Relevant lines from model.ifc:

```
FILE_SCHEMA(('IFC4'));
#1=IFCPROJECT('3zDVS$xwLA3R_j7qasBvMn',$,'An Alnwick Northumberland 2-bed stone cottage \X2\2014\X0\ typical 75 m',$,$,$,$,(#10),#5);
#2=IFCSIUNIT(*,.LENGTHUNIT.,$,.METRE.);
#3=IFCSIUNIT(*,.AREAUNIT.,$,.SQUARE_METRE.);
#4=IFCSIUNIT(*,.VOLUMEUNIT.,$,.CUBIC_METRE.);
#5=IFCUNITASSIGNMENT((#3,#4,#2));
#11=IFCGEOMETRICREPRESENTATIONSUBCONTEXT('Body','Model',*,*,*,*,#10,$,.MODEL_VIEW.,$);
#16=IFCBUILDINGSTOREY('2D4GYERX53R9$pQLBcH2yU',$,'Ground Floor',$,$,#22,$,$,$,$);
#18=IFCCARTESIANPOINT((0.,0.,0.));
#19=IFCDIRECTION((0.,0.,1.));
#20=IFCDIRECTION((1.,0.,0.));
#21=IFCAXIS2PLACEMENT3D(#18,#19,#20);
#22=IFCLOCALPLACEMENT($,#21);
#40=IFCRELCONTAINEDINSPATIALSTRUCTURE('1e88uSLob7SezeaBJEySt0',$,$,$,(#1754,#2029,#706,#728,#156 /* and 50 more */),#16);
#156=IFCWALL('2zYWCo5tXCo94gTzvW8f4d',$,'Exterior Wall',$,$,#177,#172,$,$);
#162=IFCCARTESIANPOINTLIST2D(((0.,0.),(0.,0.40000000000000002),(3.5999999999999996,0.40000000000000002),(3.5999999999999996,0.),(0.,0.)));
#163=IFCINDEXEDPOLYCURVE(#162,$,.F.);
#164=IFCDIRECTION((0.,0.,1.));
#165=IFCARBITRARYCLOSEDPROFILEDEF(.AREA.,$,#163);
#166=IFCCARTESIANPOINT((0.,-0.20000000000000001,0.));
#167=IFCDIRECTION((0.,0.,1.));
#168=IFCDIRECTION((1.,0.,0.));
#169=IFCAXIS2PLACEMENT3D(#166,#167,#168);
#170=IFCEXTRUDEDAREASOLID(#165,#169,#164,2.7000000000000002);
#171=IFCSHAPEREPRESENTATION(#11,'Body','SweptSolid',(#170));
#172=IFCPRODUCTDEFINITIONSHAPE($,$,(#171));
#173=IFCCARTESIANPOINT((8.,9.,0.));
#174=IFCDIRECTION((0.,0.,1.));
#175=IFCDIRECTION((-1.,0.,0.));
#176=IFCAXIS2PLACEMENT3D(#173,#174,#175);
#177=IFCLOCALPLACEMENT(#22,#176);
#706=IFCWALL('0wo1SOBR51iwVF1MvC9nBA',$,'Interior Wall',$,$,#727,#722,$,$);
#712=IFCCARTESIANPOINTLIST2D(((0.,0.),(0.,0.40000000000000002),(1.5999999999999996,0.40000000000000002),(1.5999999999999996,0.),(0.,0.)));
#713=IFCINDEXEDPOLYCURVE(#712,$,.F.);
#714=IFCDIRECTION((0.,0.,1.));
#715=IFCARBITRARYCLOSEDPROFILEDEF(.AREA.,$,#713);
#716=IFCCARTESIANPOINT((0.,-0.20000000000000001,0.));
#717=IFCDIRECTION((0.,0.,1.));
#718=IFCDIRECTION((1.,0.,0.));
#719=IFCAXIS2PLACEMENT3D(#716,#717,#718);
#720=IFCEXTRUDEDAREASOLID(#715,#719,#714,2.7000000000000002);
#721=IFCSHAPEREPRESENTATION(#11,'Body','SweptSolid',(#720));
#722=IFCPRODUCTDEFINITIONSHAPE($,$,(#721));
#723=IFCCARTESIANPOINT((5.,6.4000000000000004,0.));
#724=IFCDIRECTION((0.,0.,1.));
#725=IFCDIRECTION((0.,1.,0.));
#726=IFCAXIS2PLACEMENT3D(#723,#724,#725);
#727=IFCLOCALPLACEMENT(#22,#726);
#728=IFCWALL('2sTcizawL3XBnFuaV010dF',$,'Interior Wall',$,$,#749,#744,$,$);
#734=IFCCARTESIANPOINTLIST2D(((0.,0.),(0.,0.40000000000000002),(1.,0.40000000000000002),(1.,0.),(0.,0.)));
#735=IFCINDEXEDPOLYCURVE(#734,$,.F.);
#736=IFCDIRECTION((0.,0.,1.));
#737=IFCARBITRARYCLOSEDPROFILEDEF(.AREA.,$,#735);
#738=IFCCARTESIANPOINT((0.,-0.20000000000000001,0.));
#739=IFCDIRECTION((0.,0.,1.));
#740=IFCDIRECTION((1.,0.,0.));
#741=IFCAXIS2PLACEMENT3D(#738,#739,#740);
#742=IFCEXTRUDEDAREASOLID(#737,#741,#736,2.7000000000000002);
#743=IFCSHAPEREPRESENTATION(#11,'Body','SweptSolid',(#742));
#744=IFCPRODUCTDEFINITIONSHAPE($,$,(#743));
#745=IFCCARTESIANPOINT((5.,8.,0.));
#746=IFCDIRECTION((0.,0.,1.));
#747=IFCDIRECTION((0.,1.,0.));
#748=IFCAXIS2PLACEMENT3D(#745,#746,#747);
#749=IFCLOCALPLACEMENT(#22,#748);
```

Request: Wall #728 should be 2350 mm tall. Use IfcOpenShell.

```python
import ifcopenshell
import ifcopenshell.geom
import ifcopenshell.util.representation
import ifcopenshell.util.shape
import ifcopenshell.util.unit

model = ifcopenshell.open("model.ifc")
unit_scale = ifcopenshell.util.unit.calculate_unit_scale(model)
settings = ifcopenshell.geom.settings()


def volume(element):
    """Net volume in cubic metres, openings subtracted."""
    shape = ifcopenshell.geom.create_shape(settings, element)
    return ifcopenshell.util.shape.get_volume(shape.geometry)


wall = model.by_guid("2sTcizawL3XBnFuaV010dF")
before = volume(wall)

body = ifcopenshell.util.representation.get_representation(wall, "Model", "Body")
solid = body.Items[0]
old_height = solid.Depth
solid.Depth = 2.35 / unit_scale
after = volume(wall)

print(f"height {old_height:g} -> {solid.Depth:g}, volume {before:.3f} -> {after:.3f} m3")

model.write("model-out.ifc")
```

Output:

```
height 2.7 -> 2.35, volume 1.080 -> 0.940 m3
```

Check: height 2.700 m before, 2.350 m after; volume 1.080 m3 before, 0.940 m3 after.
